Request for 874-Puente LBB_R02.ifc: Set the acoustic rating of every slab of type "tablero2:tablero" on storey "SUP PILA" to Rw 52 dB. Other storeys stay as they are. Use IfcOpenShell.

First a look at what the model holds.

```python
import ifcopenshell
import ifcopenshell.util.element

model = ifcopenshell.open("874-Puente LBB_R02.ifc")
print(model.schema)
storey = next(s for s in model.by_type("IfcBuildingStorey") if s.Name == "SUP PILA")
slabs = [e for e in ifcopenshell.util.element.get_decomposition(storey) if e.is_a("IfcSlab")]
seen = {}
for e in slabs:
    element_type = ifcopenshell.util.element.get_type(e)
    key = (element_type.Name if element_type != e and element_type else None, ifcopenshell.util.element.get_pset(e, "Pset_SlabCommon", "AcousticRating"))
    seen[key] = seen.get(key, 0) + 1
for (name, value), count in sorted(seen.items(), key=str):
    print(count, "x", name, "|", value)
```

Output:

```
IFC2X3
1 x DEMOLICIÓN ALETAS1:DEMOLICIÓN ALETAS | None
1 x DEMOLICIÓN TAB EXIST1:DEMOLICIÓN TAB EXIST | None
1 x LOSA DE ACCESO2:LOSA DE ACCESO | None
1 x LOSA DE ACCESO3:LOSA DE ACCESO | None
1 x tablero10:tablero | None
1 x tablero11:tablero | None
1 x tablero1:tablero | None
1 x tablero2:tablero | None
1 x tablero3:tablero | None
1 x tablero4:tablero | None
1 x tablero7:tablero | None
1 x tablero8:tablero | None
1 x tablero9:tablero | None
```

```python
import ifcopenshell
import ifcopenshell.api.pset
import ifcopenshell.util.element

model = ifcopenshell.open("874-Puente LBB_R02.ifc")

storey = next(s for s in model.by_type("IfcBuildingStorey") if s.Name == "SUP PILA")
slabs = [e for e in ifcopenshell.util.element.get_decomposition(storey) if e.is_a("IfcSlab")]

count = 0
for e in slabs:
    element_type = ifcopenshell.util.element.get_type(e)
    if element_type in (None, e) or element_type.Name != "tablero2:tablero":
        continue
    # add_pset returns the element's existing set when there is one.
    pset = ifcopenshell.api.pset.add_pset(model, product=e, name="Pset_SlabCommon")
    ifcopenshell.api.pset.edit_pset(model, pset=pset, properties={"AcousticRating": "Rw 52 dB"})
    count += 1

print(count, "slabs updated")

model.write("874-Puente LBB_R02_updated.ifc")
```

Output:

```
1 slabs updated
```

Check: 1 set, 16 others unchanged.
